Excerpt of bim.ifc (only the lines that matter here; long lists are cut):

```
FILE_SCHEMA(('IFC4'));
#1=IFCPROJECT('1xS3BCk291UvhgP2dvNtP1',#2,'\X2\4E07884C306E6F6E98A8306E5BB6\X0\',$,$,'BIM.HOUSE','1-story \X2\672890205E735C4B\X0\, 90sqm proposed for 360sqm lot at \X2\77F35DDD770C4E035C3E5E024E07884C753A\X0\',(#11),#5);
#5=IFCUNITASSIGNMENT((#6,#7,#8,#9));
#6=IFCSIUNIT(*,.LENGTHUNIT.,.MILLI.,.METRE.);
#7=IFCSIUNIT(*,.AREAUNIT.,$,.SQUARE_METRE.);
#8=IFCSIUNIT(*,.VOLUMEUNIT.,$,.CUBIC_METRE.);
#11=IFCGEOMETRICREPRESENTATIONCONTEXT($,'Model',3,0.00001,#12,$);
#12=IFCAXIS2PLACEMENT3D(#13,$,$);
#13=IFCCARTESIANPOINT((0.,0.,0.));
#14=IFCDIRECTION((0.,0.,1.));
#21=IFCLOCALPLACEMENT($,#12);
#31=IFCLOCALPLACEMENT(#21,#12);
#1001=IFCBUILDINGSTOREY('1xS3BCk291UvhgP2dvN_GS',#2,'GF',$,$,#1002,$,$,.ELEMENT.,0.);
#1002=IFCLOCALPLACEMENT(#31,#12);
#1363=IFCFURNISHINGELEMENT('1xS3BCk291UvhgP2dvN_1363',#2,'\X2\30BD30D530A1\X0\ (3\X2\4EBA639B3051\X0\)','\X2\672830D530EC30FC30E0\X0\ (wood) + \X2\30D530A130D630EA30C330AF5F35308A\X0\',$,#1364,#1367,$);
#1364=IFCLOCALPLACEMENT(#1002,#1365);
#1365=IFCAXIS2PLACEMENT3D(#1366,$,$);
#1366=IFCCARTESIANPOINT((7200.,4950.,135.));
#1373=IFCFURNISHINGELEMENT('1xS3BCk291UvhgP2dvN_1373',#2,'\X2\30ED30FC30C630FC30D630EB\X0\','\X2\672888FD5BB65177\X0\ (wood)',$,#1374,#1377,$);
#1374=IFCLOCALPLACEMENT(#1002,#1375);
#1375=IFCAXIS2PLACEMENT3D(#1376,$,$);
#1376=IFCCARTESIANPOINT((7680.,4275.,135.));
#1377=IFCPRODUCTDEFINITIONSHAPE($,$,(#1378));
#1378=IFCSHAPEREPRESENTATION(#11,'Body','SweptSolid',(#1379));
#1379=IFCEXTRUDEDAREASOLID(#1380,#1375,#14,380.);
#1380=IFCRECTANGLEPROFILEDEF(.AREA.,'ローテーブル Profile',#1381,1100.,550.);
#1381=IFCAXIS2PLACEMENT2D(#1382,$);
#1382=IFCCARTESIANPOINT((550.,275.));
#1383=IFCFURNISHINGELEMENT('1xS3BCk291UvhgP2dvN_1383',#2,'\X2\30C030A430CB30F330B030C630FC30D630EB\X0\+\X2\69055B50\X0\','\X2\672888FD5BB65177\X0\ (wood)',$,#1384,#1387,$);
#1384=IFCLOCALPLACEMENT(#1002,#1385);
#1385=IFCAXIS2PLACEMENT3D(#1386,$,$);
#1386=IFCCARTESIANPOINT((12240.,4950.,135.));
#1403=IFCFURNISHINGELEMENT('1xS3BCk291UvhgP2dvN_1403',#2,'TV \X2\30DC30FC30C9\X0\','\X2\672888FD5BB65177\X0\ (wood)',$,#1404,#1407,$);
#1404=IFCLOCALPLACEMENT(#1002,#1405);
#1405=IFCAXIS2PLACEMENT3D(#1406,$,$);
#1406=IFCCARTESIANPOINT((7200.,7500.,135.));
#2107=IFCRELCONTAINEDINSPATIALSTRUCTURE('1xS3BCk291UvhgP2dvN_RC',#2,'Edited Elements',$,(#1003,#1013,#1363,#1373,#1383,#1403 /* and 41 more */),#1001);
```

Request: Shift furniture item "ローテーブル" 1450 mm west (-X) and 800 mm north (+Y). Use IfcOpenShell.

```python
import ifcopenshell
import ifcopenshell.api.geometry
import ifcopenshell.util.placement
import ifcopenshell.util.unit

model = ifcopenshell.open("bim.ifc")
unit_scale = ifcopenshell.util.unit.calculate_unit_scale(model)

item = model.by_guid("1xS3BCk291UvhgP2dvN_1373")
matrix = ifcopenshell.util.placement.get_local_placement(item.ObjectPlacement)
matrix[0, 3] -= 1.45 / unit_scale
matrix[1, 3] += 0.8 / unit_scale
ifcopenshell.api.geometry.edit_object_placement(model, product=item, matrix=matrix, is_si=False)

print(ifcopenshell.util.placement.get_local_placement(item.ObjectPlacement).round(3) + 0.0)

model.write("bim_rev.ifc")
```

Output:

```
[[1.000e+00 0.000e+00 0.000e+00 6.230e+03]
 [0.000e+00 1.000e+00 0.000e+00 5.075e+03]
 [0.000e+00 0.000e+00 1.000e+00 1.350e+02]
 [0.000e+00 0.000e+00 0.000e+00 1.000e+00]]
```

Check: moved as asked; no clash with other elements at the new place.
